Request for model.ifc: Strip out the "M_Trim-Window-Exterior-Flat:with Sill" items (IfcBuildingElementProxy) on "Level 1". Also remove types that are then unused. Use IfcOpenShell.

First a look at what the model holds.

```python
import ifcopenshell
import ifcopenshell.util.element

model = ifcopenshell.open("model.ifc")
print(model.schema)
storey = next(s for s in model.by_type("IfcBuildingStorey") if s.Name == "Level 1")
proxies = [e for e in ifcopenshell.util.element.get_decomposition(storey) if e.is_a("IfcBuildingElementProxy")]
seen = {}
for e in proxies:
    element_type = ifcopenshell.util.element.get_type(e)
    name = element_type.Name if element_type not in (None, e) else None
    seen[name] = seen.get(name, 0) + 1
for name, count in sorted(seen.items(), key=str):
    print(count, "x", name)
```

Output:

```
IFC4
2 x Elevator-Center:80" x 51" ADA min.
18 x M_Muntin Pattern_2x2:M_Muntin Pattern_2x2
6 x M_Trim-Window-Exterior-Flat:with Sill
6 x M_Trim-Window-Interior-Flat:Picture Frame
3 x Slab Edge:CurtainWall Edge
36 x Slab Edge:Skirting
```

```python
import ifcopenshell
import ifcopenshell.api.root
import ifcopenshell.util.element

model = ifcopenshell.open("model.ifc")

storey = next(s for s in model.by_type("IfcBuildingStorey") if s.Name == "Level 1")
proxies = [e for e in ifcopenshell.util.element.get_decomposition(storey) if e.is_a("IfcBuildingElementProxy")]
targets = [e for e in proxies if (t := ifcopenshell.util.element.get_type(e)) not in (None, e) and t.Name == "M_Trim-Window-Exterior-Flat:with Sill"]
types = {ifcopenshell.util.element.get_type(e) for e in targets} - {None, *targets}

for e in targets:
    ifcopenshell.api.root.remove_product(model, product=e)
print(len(targets), "removed")

unused = [t for t in types if not ifcopenshell.util.element.get_types(t)]
for t in unused:
    ifcopenshell.api.root.remove_product(model, product=t)
print(len(unused), "unused types removed")

model.write("model-out.ifc")
```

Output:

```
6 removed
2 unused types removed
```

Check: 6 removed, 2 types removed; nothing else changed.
